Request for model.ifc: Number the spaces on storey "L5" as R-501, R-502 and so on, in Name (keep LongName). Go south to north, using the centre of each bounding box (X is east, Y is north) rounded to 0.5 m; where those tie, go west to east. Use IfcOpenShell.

First a look at what the model holds.

```python
import ifcopenshell
import ifcopenshell.util.element
import ifcopenshell.util.placement

model = ifcopenshell.open("model.ifc")
print(model.schema)
storey = next(s for s in model.by_type("IfcBuildingStorey") if s.Name == "L5")
spaces = [e for e in ifcopenshell.util.element.get_decomposition(storey) if e.is_a("IfcSpace")]
for e in sorted(spaces, key=lambda e: e.id()):
    origin = ifcopenshell.util.placement.get_local_placement(e.ObjectPlacement)[:3, 3]
    print(e.id(), e.Name, e.LongName, origin.round(2) + 0.0, sep=" | ")
```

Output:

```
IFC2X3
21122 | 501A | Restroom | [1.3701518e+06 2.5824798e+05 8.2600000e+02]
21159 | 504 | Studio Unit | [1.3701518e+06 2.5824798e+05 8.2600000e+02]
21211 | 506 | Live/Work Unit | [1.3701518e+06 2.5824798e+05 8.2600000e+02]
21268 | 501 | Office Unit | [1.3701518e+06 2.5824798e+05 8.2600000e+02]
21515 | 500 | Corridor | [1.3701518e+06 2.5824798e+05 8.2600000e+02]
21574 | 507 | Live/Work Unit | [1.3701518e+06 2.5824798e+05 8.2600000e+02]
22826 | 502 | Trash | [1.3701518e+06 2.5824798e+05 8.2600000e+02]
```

```python
import ifcopenshell
import ifcopenshell.geom
import ifcopenshell.util.element
import ifcopenshell.util.shape

model = ifcopenshell.open("model.ifc")
settings = ifcopenshell.geom.settings()
settings.set("use-world-coords", True)


def centre(element):
    shape = ifcopenshell.geom.create_shape(settings, element)
    return ifcopenshell.util.shape.get_bbox_centroid(shape.geometry)


storey = next(s for s in model.by_type("IfcBuildingStorey") if s.Name == "L5")
spaces = [e for e in ifcopenshell.util.element.get_decomposition(storey) if e.is_a("IfcSpace")]

# Insertion points can sit at a corner or the storey origin, so sort by the geometry (in metres).
centres = {e: centre(e) for e in spaces}
spaces.sort(key=lambda e: (round(centres[e][1] / 0.5), centres[e][0]))

for i, e in enumerate(spaces, start=1):
    number = f"R-5{i:02d}"
    e.Name = number
    print(e.id(), number)

model.write("model_edited.ifc")
```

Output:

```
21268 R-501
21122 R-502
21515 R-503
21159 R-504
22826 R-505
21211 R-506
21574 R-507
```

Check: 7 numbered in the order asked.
